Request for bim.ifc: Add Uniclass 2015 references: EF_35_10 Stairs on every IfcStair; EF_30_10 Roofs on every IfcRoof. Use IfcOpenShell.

First a look at what the model holds.

```python
import ifcopenshell

model = ifcopenshell.open("bim.ifc")
print(model.schema)
print("classifications:", [c.Name for c in model.by_type("IfcClassification")])
for ifc_class in ("IfcDoor", "IfcRoof", "IfcStair", "IfcWall", "IfcWindow"):
    print(ifc_class, len(model.by_type(ifc_class)))
```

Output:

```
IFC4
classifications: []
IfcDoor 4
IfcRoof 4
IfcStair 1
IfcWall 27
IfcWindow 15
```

```python
import ifcopenshell
import ifcopenshell.api.classification

model = ifcopenshell.open("bim.ifc")

system = ifcopenshell.api.classification.add_classification(model, classification="Uniclass 2015")

codes = {
    "IfcStair": ("EF_35_10", "Stairs"),
    "IfcRoof": ("EF_30_10", "Roofs"),
}
for ifc_class, (code, name) in codes.items():
    products = model.by_type(ifc_class)
    ifcopenshell.api.classification.add_reference(
        model, products=products, classification=system, identification=code, name=name
    )
    print(code, len(products))

model.write("bim_edited.ifc")
```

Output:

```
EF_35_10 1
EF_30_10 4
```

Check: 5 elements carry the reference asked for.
